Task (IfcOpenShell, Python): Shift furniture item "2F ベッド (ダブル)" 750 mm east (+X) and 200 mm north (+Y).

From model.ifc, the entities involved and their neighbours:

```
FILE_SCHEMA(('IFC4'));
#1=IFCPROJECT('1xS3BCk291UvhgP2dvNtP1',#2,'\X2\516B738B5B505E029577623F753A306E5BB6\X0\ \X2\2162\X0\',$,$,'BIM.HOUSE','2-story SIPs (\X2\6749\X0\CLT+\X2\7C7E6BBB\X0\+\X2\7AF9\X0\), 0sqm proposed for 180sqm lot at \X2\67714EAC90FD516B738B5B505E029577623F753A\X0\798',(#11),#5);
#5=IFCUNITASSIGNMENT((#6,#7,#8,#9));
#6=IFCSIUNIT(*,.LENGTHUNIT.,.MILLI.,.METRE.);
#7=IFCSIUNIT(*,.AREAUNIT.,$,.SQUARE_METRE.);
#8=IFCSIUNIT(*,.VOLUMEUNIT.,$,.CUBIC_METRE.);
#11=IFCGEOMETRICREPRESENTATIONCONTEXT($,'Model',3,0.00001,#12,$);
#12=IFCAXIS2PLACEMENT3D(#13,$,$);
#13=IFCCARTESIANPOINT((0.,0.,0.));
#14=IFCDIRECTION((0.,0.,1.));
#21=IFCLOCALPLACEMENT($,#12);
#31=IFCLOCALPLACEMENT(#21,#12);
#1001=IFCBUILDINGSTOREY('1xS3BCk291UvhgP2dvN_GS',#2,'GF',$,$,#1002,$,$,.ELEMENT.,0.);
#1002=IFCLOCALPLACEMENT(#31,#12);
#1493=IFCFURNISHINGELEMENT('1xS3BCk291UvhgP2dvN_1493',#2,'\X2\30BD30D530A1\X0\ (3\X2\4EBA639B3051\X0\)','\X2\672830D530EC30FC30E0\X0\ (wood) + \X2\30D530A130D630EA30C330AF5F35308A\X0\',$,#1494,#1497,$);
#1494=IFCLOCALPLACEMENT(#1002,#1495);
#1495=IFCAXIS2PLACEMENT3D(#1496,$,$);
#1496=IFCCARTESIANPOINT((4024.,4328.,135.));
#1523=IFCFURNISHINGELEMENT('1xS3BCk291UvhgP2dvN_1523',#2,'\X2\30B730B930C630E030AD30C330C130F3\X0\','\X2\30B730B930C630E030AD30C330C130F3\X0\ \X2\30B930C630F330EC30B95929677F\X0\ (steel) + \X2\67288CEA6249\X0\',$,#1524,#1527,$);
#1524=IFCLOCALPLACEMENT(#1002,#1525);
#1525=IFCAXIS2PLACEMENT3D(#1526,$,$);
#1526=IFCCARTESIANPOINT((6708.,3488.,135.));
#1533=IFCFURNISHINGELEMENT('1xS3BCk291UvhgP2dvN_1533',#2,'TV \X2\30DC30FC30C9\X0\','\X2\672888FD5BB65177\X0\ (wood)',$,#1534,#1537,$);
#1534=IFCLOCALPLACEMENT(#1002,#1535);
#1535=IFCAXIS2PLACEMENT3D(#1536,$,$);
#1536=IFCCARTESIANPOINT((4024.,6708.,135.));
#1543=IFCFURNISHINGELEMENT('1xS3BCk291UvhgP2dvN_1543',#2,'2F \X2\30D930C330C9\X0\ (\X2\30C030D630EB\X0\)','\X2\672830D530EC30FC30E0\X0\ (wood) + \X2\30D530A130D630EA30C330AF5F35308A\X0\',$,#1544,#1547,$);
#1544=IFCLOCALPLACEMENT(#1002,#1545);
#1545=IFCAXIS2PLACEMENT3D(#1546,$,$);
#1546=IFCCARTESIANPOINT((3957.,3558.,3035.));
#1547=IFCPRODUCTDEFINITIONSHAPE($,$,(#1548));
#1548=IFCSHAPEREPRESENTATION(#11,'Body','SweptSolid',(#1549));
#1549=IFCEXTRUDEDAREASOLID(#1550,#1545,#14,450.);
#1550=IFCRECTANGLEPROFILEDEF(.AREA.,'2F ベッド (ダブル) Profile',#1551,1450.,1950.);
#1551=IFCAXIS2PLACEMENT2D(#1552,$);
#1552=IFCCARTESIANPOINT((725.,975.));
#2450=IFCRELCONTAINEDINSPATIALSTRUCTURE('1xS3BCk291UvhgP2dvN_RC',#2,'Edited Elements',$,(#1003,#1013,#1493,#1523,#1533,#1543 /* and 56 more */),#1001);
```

```python
import ifcopenshell
import ifcopenshell.api.geometry
import ifcopenshell.util.placement
import ifcopenshell.util.unit

model = ifcopenshell.open("model.ifc")
unit_scale = ifcopenshell.util.unit.calculate_unit_scale(model)

item = model.by_guid("1xS3BCk291UvhgP2dvN_1543")
matrix = ifcopenshell.util.placement.get_local_placement(item.ObjectPlacement)
matrix[0, 3] += 0.75 / unit_scale
matrix[1, 3] += 0.2 / unit_scale
ifcopenshell.api.geometry.edit_object_placement(model, product=item, matrix=matrix, is_si=False)

print(ifcopenshell.util.placement.get_local_placement(item.ObjectPlacement).round(3) + 0.0)

model.write("model_rev.ifc")
```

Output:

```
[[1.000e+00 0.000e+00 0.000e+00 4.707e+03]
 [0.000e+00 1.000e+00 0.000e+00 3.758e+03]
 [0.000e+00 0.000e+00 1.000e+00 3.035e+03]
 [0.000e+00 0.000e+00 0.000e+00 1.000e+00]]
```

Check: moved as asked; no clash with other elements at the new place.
